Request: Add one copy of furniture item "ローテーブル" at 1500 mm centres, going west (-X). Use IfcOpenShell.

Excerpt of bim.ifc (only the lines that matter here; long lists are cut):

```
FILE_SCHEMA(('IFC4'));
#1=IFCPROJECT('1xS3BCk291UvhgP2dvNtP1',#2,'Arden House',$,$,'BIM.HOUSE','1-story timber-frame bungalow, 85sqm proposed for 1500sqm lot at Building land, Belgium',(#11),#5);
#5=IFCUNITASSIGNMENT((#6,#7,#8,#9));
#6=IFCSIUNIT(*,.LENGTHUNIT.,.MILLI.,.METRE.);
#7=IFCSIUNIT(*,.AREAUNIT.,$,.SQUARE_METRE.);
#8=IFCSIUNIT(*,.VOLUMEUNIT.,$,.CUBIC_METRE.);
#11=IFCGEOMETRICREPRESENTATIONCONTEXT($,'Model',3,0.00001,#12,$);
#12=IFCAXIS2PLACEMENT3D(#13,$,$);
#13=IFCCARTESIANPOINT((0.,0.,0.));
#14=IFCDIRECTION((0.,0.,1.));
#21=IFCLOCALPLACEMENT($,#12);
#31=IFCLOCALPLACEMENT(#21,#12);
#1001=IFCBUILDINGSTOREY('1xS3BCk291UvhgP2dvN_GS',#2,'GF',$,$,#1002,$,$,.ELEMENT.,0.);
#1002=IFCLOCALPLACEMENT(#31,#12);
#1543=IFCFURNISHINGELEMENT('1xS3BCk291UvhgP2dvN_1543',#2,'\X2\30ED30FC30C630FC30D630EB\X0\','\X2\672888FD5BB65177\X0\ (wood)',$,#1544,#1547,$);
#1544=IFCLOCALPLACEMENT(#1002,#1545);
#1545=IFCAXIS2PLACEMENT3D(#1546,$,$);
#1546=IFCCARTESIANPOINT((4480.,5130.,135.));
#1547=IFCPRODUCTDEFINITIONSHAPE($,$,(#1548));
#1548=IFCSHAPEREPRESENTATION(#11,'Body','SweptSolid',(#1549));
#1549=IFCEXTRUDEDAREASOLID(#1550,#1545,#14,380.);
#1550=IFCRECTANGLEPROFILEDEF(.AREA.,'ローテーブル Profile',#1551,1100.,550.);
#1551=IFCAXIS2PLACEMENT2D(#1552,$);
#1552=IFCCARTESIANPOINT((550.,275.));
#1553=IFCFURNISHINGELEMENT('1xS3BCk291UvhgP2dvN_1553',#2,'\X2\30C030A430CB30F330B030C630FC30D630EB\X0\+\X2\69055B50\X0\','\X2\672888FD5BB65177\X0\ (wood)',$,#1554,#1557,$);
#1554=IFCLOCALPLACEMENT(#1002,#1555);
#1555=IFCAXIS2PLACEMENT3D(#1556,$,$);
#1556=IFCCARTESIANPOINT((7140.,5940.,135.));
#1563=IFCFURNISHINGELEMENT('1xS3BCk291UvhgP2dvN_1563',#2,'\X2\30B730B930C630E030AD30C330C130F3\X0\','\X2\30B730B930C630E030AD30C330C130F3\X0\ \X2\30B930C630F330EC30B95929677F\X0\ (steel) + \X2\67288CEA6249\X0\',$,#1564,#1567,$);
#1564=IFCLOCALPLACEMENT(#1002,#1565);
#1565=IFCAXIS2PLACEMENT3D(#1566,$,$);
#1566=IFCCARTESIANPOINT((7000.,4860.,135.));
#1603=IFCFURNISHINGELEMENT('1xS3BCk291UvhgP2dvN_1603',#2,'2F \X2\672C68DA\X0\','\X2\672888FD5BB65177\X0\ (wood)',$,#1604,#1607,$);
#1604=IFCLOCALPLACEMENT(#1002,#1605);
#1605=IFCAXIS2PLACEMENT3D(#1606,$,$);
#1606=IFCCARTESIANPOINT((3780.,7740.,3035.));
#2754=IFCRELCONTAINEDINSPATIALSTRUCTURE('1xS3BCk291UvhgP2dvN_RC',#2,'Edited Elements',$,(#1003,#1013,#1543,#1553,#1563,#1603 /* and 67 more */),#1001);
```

```python
import numpy as np
import ifcopenshell
import ifcopenshell.api.geometry
import ifcopenshell.api.root
import ifcopenshell.util.element
import ifcopenshell.util.placement
import ifcopenshell.util.unit

model = ifcopenshell.open("bim.ifc")
unit_scale = ifcopenshell.util.unit.calculate_unit_scale(model)


def reuse_history(source, copy):
    """copy_class also copies each property set's owner history, people and application; keep the originals."""
    for rel in copy.IsDefinedBy:
        if rel.is_a("IfcRelDefinesByProperties") and (history := rel.RelatingPropertyDefinition.OwnerHistory):
            rel.RelatingPropertyDefinition.OwnerHistory = source.OwnerHistory
            ifcopenshell.util.element.remove_deep2(model, history)


source = model.by_id(1543)
base = ifcopenshell.util.placement.get_local_placement(source.ObjectPlacement)
step = np.array([-1.0, 0.0, 0.0]) * 1.5 / unit_scale

for i in range(1, 2):
    copy = ifcopenshell.api.root.copy_class(model, product=source)
    copy.Representation = ifcopenshell.util.element.copy_deep(
        model, source.Representation, exclude=["IfcGeometricRepresentationContext", "IfcRepresentationMap"]
    )
    reuse_history(source, copy)
    matrix = base.copy()
    matrix[:3, 3] += i * step
    print("added at", matrix[:3, 3].round(3) + 0.0)
    ifcopenshell.api.geometry.edit_object_placement(model, product=copy, matrix=matrix, is_si=False)

model.write("bim_edited.ifc")
```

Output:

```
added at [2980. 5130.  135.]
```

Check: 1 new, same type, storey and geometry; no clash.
